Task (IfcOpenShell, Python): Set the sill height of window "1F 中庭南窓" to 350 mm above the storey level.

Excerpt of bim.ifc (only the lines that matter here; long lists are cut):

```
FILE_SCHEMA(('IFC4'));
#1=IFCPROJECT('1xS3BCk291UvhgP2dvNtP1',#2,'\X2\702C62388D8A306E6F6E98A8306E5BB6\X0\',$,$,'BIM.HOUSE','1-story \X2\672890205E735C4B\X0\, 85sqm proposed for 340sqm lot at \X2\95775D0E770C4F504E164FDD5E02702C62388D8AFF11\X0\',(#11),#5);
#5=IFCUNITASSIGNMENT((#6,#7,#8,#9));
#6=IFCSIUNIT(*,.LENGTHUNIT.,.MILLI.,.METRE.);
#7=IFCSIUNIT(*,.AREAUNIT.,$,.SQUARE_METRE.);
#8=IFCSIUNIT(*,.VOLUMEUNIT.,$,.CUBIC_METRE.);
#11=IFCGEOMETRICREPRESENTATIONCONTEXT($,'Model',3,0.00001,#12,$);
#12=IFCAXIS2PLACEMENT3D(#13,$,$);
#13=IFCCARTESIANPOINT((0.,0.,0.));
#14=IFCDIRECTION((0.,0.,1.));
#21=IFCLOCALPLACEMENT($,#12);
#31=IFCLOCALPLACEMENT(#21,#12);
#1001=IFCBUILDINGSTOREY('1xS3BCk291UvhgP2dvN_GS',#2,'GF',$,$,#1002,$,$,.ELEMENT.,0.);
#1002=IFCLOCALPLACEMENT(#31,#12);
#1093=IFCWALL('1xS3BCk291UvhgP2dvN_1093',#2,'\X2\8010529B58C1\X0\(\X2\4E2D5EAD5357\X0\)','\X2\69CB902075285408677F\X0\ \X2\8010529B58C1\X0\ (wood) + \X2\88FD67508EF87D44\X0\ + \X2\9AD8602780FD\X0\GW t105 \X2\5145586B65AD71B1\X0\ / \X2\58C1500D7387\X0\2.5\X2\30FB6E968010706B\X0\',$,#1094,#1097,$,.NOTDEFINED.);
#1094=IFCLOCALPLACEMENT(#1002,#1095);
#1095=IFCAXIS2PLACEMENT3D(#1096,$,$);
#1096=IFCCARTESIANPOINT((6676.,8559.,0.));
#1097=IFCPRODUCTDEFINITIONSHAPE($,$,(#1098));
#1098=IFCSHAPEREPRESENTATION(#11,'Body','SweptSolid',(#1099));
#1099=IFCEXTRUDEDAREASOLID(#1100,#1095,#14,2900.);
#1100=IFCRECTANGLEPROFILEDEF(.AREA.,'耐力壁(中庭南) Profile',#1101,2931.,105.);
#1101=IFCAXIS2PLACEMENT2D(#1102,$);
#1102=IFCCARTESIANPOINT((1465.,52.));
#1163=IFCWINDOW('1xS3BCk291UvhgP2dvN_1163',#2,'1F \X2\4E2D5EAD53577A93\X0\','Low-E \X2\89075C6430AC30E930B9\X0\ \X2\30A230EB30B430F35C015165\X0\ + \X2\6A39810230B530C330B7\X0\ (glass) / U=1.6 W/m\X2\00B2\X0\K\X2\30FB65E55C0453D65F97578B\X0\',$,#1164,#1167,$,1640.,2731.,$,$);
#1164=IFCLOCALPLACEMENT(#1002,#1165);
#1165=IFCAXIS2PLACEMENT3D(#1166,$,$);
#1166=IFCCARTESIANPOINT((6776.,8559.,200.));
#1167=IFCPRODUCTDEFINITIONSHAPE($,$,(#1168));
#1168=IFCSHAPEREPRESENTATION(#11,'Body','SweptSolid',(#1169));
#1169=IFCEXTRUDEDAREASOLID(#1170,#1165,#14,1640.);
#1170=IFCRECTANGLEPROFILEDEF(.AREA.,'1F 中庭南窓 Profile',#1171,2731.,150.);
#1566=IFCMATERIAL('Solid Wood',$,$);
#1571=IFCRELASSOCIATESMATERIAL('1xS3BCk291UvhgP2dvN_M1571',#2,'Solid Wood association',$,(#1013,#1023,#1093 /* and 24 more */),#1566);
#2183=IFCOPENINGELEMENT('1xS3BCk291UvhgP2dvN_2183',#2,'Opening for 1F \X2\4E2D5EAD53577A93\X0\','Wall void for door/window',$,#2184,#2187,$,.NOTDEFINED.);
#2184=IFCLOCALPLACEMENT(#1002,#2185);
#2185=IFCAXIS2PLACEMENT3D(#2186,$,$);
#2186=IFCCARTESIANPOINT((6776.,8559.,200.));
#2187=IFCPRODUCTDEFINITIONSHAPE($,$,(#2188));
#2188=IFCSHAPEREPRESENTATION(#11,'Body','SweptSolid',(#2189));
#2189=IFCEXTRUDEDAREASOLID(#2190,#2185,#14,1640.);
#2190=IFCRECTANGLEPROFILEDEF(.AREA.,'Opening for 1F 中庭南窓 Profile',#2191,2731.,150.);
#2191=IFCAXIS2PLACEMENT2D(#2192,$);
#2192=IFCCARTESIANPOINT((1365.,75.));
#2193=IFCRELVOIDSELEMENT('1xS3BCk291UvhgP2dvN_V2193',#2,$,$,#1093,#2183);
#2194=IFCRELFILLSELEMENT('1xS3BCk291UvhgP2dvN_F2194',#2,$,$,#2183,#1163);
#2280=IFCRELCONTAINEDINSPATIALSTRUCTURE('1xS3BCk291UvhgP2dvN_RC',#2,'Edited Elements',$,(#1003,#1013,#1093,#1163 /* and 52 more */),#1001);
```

```python
import numpy as np
import ifcopenshell
import ifcopenshell.api.geometry
import ifcopenshell.geom
import ifcopenshell.util.element
import ifcopenshell.util.placement
import ifcopenshell.util.shape
import ifcopenshell.util.unit

model = ifcopenshell.open("bim.ifc")
unit_scale = ifcopenshell.util.unit.calculate_unit_scale(model)

window = model.by_id(1163)
opening = window.FillsVoids[0].RelatingOpeningElement
storey = ifcopenshell.util.element.get_container(window, ifc_class="IfcBuildingStorey")
level = ifcopenshell.util.placement.get_local_placement(storey.ObjectPlacement)[2, 3]

# The opening's origin need not be at the sill, so measure its lowest point.
shape = ifcopenshell.geom.create_shape(ifcopenshell.geom.settings(), opening)
bottom = ifcopenshell.util.shape.get_shape_bottom_elevation(shape, shape.geometry) / unit_scale
dz = level + 350.0 - bottom

shift = np.array([0.0, 0.0, dz])
# The window is not placed relative to its opening, so move both.
for product in (opening, window):
    matrix = ifcopenshell.util.placement.get_local_placement(product.ObjectPlacement)
    matrix[:3, 3] += shift
    ifcopenshell.api.geometry.edit_object_placement(model, product=product, matrix=matrix, is_si=False)

print(f"moved by {dz * unit_scale:+.3f} m")

model.write("bim-out.ifc")
```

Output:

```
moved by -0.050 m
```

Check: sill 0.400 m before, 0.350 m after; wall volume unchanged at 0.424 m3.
